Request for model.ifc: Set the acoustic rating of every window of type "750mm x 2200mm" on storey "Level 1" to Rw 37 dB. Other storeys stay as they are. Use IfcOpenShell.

First a look at what the model holds.

```python
import ifcopenshell
import ifcopenshell.util.element

model = ifcopenshell.open("model.ifc")
print(model.schema)
storey = next(s for s in model.by_type("IfcBuildingStorey") if s.Name == "Level 1")
windows = [e for e in ifcopenshell.util.element.get_decomposition(storey) if e.is_a("IfcWindow")]
seen = {}
for e in windows:
    element_type = ifcopenshell.util.element.get_type(e)
    key = (element_type.Name if element_type != e and element_type else None, ifcopenshell.util.element.get_pset(e, "Pset_WindowCommon", "AcousticRating"))
    seen[key] = seen.get(key, 0) + 1
for (name, value), count in sorted(seen.items(), key=str):
    print(count, "x", name, "|", value)
```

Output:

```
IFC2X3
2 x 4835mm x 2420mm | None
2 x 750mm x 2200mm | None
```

```python
import ifcopenshell
import ifcopenshell.api.pset
import ifcopenshell.util.element

model = ifcopenshell.open("model.ifc")

storey = next(s for s in model.by_type("IfcBuildingStorey") if s.Name == "Level 1")
windows = [e for e in ifcopenshell.util.element.get_decomposition(storey) if e.is_a("IfcWindow")]

count = 0
for e in windows:
    element_type = ifcopenshell.util.element.get_type(e)
    if element_type in (None, e) or element_type.Name != "750mm x 2200mm":
        continue
    # add_pset returns the element's existing set when there is one.
    pset = ifcopenshell.api.pset.add_pset(model, product=e, name="Pset_WindowCommon")
    ifcopenshell.api.pset.edit_pset(model, pset=pset, properties={"AcousticRating": "Rw 37 dB"})
    count += 1

print(count, "windows updated")

model.write("model_edited.ifc")
```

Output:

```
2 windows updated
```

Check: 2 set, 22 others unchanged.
